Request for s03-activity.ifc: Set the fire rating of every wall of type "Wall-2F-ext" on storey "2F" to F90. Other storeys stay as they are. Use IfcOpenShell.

First a look at what the model holds.

```python
import ifcopenshell
import ifcopenshell.util.element

model = ifcopenshell.open("s03-activity.ifc")
print(model.schema)
storey = next(s for s in model.by_type("IfcBuildingStorey") if s.Name == "2F")
walls = [e for e in ifcopenshell.util.element.get_decomposition(storey) if e.is_a("IfcWall")]
seen = {}
for e in walls:
    element_type = ifcopenshell.util.element.get_type(e)
    key = (element_type.Name if element_type != e and element_type else None, ifcopenshell.util.element.get_pset(e, "Pset_WallCommon", "FireRating"))
    seen[key] = seen.get(key, 0) + 1
for (name, value), count in sorted(seen.items(), key=str):
    print(count, "x", name, "|", value)
```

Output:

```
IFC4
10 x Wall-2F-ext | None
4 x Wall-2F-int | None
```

```python
import ifcopenshell
import ifcopenshell.api.pset
import ifcopenshell.util.element

model = ifcopenshell.open("s03-activity.ifc")

storey = next(s for s in model.by_type("IfcBuildingStorey") if s.Name == "2F")
walls = [e for e in ifcopenshell.util.element.get_decomposition(storey) if e.is_a("IfcWall")]

count = 0
for e in walls:
    element_type = ifcopenshell.util.element.get_type(e)
    if element_type in (None, e) or element_type.Name != "Wall-2F-ext":
        continue
    # add_pset returns the element's existing set when there is one.
    pset = ifcopenshell.api.pset.add_pset(model, product=e, name="Pset_WallCommon")
    ifcopenshell.api.pset.edit_pset(model, pset=pset, properties={"FireRating": "F90"})
    count += 1

print(count, "walls updated")

model.write("s03-activity_edited.ifc")
```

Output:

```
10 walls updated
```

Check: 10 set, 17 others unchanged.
